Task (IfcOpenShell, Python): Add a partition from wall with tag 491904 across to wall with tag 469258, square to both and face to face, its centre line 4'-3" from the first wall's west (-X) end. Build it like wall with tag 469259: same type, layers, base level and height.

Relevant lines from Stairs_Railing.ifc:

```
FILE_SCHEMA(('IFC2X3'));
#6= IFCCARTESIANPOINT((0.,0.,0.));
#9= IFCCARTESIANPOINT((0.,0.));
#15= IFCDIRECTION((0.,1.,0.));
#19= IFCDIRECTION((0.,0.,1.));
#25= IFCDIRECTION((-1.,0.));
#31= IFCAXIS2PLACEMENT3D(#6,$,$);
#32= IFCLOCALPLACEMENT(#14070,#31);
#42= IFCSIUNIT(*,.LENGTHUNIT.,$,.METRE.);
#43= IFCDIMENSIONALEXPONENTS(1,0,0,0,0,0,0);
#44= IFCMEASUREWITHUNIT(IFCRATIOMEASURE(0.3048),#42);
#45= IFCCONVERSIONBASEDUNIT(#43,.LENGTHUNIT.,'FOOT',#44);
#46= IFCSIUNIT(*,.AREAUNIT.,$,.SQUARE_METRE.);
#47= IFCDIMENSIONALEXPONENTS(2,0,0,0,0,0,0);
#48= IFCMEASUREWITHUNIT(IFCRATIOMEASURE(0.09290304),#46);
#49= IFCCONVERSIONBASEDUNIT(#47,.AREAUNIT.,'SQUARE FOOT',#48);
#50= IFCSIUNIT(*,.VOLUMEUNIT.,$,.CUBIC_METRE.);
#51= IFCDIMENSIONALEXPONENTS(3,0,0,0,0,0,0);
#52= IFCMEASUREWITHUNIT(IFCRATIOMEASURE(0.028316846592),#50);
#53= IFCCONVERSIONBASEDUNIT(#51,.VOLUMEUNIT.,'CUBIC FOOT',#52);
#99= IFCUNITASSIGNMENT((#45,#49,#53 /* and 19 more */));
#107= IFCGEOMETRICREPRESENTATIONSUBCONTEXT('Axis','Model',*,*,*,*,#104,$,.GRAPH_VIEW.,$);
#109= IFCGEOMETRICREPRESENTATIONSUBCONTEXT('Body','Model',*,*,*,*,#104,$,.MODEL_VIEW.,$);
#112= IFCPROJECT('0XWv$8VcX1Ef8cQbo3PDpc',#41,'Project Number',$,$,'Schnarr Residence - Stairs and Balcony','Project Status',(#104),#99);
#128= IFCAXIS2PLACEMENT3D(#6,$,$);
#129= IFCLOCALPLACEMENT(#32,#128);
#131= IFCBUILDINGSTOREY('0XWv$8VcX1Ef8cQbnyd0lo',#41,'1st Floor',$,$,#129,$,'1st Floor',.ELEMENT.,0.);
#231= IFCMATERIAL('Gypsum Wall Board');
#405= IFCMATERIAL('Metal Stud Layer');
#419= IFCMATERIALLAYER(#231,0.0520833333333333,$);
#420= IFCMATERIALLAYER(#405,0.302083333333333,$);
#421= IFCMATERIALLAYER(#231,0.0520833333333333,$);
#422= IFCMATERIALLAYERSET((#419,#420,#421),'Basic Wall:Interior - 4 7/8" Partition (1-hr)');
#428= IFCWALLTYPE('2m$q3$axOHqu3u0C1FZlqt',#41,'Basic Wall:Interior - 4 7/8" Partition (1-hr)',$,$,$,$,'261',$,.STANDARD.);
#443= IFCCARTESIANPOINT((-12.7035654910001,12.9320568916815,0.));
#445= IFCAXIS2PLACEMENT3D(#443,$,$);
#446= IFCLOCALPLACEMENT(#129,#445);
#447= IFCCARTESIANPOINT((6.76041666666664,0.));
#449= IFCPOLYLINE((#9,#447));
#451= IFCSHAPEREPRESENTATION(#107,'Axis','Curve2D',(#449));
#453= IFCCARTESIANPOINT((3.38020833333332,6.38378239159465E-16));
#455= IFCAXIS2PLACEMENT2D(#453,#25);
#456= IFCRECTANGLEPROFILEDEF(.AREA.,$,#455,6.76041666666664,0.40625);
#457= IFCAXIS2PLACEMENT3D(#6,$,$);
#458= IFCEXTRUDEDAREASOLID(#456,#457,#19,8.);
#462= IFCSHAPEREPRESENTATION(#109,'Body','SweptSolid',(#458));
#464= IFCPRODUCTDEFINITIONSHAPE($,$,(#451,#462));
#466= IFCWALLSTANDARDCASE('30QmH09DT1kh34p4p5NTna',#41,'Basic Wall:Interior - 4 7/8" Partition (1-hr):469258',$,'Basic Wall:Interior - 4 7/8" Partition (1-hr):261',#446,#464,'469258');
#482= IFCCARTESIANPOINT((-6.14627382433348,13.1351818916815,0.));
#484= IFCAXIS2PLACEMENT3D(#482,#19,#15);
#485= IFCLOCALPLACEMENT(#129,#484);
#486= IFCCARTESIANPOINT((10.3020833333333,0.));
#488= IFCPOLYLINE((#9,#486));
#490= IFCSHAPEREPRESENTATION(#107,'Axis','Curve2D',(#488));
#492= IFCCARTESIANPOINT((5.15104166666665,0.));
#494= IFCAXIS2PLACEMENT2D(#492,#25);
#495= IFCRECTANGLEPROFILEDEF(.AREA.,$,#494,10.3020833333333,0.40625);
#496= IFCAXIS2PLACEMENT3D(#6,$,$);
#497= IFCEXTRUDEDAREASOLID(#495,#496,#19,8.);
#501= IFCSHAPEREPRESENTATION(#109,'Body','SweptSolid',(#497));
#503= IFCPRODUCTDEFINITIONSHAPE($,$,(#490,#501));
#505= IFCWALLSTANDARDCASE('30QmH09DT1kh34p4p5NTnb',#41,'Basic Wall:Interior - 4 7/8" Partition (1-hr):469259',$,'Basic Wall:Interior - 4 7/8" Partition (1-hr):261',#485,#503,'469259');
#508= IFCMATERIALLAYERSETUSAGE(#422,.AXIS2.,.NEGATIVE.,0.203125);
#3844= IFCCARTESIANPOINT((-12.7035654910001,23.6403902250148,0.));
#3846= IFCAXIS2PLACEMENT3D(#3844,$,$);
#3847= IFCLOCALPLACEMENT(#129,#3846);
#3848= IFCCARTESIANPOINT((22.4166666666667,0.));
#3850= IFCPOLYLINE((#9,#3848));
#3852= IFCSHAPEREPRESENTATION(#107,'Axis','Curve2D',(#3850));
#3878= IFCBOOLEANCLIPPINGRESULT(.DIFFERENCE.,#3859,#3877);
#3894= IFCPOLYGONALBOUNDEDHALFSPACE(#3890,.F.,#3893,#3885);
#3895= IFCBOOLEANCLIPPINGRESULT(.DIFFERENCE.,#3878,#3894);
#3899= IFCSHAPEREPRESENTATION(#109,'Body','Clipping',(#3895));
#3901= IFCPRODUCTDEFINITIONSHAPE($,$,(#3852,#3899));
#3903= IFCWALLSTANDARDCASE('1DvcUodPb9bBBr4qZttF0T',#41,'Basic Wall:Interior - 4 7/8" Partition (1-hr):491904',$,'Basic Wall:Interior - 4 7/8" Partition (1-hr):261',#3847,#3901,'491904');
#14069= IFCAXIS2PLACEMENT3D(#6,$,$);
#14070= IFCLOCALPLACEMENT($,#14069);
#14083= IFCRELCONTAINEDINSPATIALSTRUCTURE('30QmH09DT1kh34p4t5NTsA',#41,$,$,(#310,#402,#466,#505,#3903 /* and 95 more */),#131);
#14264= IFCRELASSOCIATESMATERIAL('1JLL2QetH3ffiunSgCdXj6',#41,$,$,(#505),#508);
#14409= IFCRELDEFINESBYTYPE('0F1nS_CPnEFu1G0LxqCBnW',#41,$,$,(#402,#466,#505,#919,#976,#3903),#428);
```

```python
import numpy as np
import ifcopenshell
import ifcopenshell.api.geometry
import ifcopenshell.api.material
import ifcopenshell.api.pset
import ifcopenshell.api.root
import ifcopenshell.api.spatial
import ifcopenshell.api.type
import ifcopenshell.geom
import ifcopenshell.util.element
import ifcopenshell.util.placement
import ifcopenshell.util.representation
import ifcopenshell.util.shape
import ifcopenshell.util.unit

model = ifcopenshell.open("Stairs_Railing.ifc")
unit_scale = ifcopenshell.util.unit.calculate_unit_scale(model)
settings = ifcopenshell.geom.settings()
settings.set("use-world-coords", True)

start_wall = model.by_guid("1DvcUodPb9bBBr4qZttF0T")
end_wall = model.by_guid("30QmH09DT1kh34p4p5NTna")
like = model.by_guid("30QmH09DT1kh34p4p5NTnb")
matrix = ifcopenshell.util.placement.get_local_placement(start_wall.ObjectPlacement)
matrix[:3, 3] *= unit_scale


def extent(element):
    """Bounding box in the first wall's axes, in metres."""
    shape = ifcopenshell.geom.create_shape(settings, element)
    points = (ifcopenshell.util.shape.get_vertices(shape.geometry) - matrix[:3, 3]) @ matrix[:3, :3]
    return points.min(axis=0), points.max(axis=0)


y_start = extent(start_wall)[0][1]
y_end = extent(end_wall)[1][1]
like_min, like_max = extent(like)
length, height = float(abs(y_end - y_start)), float(like_max[2] - like_min[2])
layer_set = ifcopenshell.util.element.get_material(like, should_skip_usage=True)
thickness = sum(layer.LayerThickness for layer in layer_set.MaterialLayers) * unit_scale

wall = ifcopenshell.api.root.create_entity(model, ifc_class="IfcWallStandardCase", name="New partition")
storey = ifcopenshell.util.element.get_container(like)
ifcopenshell.api.spatial.assign_container(model, products=[wall], relating_structure=storey)
ifcopenshell.api.type.assign_type(
    model, related_objects=[wall], relating_type=ifcopenshell.util.element.get_type(like), should_map_representations=False
)
rel = ifcopenshell.api.material.assign_material(
    model, products=[wall], type="IfcMaterialLayerSetUsage", material=layer_set
)
rel.RelatingMaterial.OffsetFromReferenceLine = -thickness / 2 / unit_scale
pset = ifcopenshell.api.pset.add_pset(model, product=wall, name="Pset_WallCommon")
ifcopenshell.api.pset.edit_pset(model, pset=pset, properties={"IsExternal": False, "LoadBearing": False})

# The axis runs down the middle of the wall.
axis = ifcopenshell.api.geometry.add_axis_representation(
    model, context=ifcopenshell.util.representation.get_context(model, "Model", "Axis"), axis=[(0.0, 0.0), (length, 0.0)]
)
body = ifcopenshell.api.geometry.add_wall_representation(
    model,
    context=ifcopenshell.util.representation.get_context(model, "Model", "Body", "MODEL_VIEW"),
    length=length,
    height=height,
    thickness=thickness,
    offset=-thickness / 2,
)
for representation in (axis, body):
    ifcopenshell.api.geometry.assign_representation(model, product=wall, representation=representation)

placement = matrix @ ifcopenshell.util.placement.rotation(-90, "Z")
placement[:, 3] = matrix @ np.array([extent(start_wall)[0][0] + 1.2954, y_start, like_min[2], 1.0])
ifcopenshell.api.geometry.edit_object_placement(model, product=wall, matrix=placement)

print(f"partition {length:.3f} m long, {height:.3f} m high, {thickness:.3f} m thick")

model.write("Stairs_Railing_edited.ifc")
```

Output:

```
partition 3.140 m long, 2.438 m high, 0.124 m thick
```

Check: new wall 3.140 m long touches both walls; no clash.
